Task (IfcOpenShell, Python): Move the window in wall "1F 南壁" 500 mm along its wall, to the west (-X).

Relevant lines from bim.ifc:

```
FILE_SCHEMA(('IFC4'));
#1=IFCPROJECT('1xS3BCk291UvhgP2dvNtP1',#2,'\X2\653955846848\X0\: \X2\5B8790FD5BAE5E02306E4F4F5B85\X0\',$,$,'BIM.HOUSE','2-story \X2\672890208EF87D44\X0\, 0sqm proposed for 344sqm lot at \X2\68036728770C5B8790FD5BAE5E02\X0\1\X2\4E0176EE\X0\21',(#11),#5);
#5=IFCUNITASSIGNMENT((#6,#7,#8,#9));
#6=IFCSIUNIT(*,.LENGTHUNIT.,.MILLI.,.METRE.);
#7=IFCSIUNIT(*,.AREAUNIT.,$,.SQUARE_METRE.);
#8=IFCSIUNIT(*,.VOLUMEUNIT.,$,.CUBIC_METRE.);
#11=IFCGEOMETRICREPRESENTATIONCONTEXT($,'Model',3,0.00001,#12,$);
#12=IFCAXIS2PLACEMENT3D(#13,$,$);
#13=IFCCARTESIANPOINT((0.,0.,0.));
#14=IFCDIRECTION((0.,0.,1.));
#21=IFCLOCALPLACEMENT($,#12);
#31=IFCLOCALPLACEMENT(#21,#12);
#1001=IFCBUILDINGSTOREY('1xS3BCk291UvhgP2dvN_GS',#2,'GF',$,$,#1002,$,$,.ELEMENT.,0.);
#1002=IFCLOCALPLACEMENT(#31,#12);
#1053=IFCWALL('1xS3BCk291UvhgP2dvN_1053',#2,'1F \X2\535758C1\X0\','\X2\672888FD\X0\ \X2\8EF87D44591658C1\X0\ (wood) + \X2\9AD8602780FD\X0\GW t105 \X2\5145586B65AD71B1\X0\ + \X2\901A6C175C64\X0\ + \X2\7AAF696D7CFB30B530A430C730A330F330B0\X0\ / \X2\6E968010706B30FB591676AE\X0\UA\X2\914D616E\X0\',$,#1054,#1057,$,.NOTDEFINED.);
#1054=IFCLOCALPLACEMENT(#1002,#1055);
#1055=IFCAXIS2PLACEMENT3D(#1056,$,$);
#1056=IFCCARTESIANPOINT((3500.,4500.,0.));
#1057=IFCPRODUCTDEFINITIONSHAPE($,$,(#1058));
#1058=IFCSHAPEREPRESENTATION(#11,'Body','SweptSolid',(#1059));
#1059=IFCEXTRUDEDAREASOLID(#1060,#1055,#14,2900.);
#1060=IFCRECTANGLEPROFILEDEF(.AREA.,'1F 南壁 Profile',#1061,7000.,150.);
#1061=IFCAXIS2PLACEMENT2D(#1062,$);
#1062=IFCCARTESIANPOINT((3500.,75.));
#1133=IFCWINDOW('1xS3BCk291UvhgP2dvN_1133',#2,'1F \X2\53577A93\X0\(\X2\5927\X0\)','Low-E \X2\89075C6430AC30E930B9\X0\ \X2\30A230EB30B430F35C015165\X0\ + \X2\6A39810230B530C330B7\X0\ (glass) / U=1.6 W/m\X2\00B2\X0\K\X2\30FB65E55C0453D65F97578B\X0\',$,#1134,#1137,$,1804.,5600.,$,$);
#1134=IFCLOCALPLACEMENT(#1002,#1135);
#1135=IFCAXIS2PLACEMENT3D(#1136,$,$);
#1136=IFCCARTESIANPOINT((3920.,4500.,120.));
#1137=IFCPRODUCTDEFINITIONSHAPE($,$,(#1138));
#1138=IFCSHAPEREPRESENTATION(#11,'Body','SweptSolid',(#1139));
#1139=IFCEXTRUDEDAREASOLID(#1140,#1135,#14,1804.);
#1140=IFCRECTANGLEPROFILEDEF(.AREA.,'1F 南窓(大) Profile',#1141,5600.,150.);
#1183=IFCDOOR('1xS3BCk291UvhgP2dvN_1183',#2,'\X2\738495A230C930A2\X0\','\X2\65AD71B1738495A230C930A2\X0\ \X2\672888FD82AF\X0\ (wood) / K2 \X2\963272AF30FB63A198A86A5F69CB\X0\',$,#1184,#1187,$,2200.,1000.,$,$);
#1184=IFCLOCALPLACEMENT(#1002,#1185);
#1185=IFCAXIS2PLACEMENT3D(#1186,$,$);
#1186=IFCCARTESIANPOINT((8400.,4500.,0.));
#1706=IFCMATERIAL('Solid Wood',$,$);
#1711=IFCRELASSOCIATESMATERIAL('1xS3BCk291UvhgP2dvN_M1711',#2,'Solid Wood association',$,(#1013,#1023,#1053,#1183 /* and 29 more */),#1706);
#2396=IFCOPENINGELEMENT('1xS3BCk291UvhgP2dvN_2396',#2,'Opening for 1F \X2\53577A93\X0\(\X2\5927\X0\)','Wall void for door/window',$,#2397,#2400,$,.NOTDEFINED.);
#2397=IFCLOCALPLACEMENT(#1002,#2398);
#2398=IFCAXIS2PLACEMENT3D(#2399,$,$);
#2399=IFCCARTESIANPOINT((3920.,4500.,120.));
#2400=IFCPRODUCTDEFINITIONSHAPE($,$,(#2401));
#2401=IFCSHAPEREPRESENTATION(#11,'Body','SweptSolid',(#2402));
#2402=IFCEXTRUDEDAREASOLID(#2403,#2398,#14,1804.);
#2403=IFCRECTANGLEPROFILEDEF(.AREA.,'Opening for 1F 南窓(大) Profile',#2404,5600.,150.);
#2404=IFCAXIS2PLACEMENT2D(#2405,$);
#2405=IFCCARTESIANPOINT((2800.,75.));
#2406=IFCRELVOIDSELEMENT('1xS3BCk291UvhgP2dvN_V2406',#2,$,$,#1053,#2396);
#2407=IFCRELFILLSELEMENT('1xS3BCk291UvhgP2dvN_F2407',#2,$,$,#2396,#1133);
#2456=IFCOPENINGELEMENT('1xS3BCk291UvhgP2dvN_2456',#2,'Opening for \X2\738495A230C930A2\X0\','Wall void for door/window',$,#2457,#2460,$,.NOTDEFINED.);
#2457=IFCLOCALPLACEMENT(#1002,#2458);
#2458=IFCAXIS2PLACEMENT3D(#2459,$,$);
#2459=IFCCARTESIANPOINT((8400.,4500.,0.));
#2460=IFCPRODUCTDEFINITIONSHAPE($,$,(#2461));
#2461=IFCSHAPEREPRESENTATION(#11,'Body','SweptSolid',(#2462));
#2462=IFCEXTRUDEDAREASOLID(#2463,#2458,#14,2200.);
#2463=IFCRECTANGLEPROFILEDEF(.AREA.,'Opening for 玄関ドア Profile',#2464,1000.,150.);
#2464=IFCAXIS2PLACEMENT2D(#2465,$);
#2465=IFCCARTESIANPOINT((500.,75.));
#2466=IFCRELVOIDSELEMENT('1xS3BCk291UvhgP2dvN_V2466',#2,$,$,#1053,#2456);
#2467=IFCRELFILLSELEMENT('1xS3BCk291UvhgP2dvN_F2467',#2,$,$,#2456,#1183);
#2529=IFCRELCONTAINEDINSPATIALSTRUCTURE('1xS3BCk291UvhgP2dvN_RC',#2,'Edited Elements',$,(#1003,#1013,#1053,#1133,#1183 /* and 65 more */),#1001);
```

```python
import ifcopenshell
import ifcopenshell.api.geometry
import ifcopenshell.util.placement
import ifcopenshell.util.unit

model = ifcopenshell.open("bim.ifc")
unit_scale = ifcopenshell.util.unit.calculate_unit_scale(model)

window = model.by_guid("1xS3BCk291UvhgP2dvN_1133")
opening = window.FillsVoids[0].RelatingOpeningElement
wall = opening.VoidsElements[0].RelatingBuildingElement

wall_matrix = ifcopenshell.util.placement.get_local_placement(wall.ObjectPlacement)
shift = wall_matrix[:3, 0] * -0.5 / unit_scale
before = ifcopenshell.util.placement.get_local_placement(window.ObjectPlacement)[:3, 3].copy()

# The window is not placed relative to its opening, so move both.
for product in (opening, window):
    matrix = ifcopenshell.util.placement.get_local_placement(product.ObjectPlacement)
    matrix[:3, 3] += shift
    ifcopenshell.api.geometry.edit_object_placement(model, product=product, matrix=matrix, is_si=False)

after = ifcopenshell.util.placement.get_local_placement(window.ObjectPlacement)[:3, 3]
print("window moved by", (after - before).round(3) + 0.0)

model.write("bim_updated.ifc")
```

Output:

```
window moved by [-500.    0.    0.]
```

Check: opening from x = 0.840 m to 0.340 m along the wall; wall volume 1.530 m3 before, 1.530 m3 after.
